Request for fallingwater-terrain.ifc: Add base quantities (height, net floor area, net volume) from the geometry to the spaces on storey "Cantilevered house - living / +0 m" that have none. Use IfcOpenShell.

First a look at what the model holds.

```python
import ifcopenshell
import ifcopenshell.util.element
import ifcopenshell.util.unit

model = ifcopenshell.open("fallingwater-terrain.ifc")
print(model.schema)
for unit_type in ("LENGTHUNIT", "AREAUNIT", "VOLUMEUNIT"):
    print(unit_type, ifcopenshell.util.unit.calculate_unit_scale(model, unit_type))
storey = next(s for s in model.by_type("IfcBuildingStorey") if s.Name == "Cantilevered house - living / +0 m")
spaces = [e for e in ifcopenshell.util.element.get_decomposition(storey) if e.is_a("IfcSpace")]
for e in sorted(spaces, key=lambda e: e.id()):
    print(e.id(), e.is_a(), e.Name, list(ifcopenshell.util.element.get_psets(e, qtos_only=True)), sep=" | ")
```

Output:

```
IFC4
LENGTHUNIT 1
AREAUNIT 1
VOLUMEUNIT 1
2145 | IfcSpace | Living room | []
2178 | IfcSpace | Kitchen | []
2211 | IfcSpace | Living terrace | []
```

```python
import ifcopenshell
import ifcopenshell.api.pset
import ifcopenshell.geom
import ifcopenshell.util.element
import ifcopenshell.util.shape
import ifcopenshell.util.unit

model = ifcopenshell.open("fallingwater-terrain.ifc")
unit_scale = ifcopenshell.util.unit.calculate_unit_scale(model)
area_scale = ifcopenshell.util.unit.calculate_unit_scale(model, "AREAUNIT")
volume_scale = ifcopenshell.util.unit.calculate_unit_scale(model, "VOLUMEUNIT")
settings = ifcopenshell.geom.settings()

storey = next(s for s in model.by_type("IfcBuildingStorey") if s.Name == "Cantilevered house - living / +0 m")
spaces = [e for e in ifcopenshell.util.element.get_decomposition(storey) if e.is_a("IfcSpace")]

for e in sorted(spaces, key=lambda e: e.id()):
    if ifcopenshell.util.element.get_psets(e, qtos_only=True, should_inherit=False):
        continue
    # Geometry comes back in metres, in the element's own axes.
    shape = ifcopenshell.geom.create_shape(settings, e)
    values = {
        "Height": ifcopenshell.util.shape.get_z(shape.geometry) / unit_scale,
        "NetFloorArea": ifcopenshell.util.shape.get_footprint_area(shape.geometry) / area_scale,
        "NetVolume": ifcopenshell.util.shape.get_volume(shape.geometry) / volume_scale,
    }
    qto = ifcopenshell.api.pset.add_qto(model, product=e, name="Qto_SpaceBaseQuantities")
    ifcopenshell.api.pset.edit_qto(model, qto=qto, properties=values)
    print(e.id(), {k: round(v, 3) for k, v in values.items()})

model.write("fallingwater-terrain_edited.ifc")
```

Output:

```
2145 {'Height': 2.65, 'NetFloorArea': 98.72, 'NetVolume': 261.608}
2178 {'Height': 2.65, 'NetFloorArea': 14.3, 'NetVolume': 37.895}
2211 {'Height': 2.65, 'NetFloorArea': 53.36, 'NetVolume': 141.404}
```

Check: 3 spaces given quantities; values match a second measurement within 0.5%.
